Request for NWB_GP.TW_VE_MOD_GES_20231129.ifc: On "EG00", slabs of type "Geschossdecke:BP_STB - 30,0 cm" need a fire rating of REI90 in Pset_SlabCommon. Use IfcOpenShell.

First a look at what the model holds.

```python
import ifcopenshell
import ifcopenshell.util.element

model = ifcopenshell.open("NWB_GP.TW_VE_MOD_GES_20231129.ifc")
print(model.schema)
storey = next(s for s in model.by_type("IfcBuildingStorey") if s.Name == "EG00")
slabs = [e for e in ifcopenshell.util.element.get_decomposition(storey) if e.is_a("IfcSlab")]
seen = {}
for e in slabs:
    element_type = ifcopenshell.util.element.get_type(e)
    key = (element_type.Name if element_type != e and element_type else None, ifcopenshell.util.element.get_pset(e, "Pset_SlabCommon", "FireRating"))
    seen[key] = seen.get(key, 0) + 1
for (name, value), count in sorted(seen.items(), key=str):
    print(count, "x", name, "|", value)
```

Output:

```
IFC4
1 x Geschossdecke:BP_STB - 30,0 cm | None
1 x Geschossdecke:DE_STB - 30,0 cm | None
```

```python
import ifcopenshell
import ifcopenshell.api.pset
import ifcopenshell.util.element

model = ifcopenshell.open("NWB_GP.TW_VE_MOD_GES_20231129.ifc")

storey = next(s for s in model.by_type("IfcBuildingStorey") if s.Name == "EG00")
slabs = [e for e in ifcopenshell.util.element.get_decomposition(storey) if e.is_a("IfcSlab")]

count = 0
for e in slabs:
    element_type = ifcopenshell.util.element.get_type(e)
    if element_type in (None, e) or element_type.Name != "Geschossdecke:BP_STB - 30,0 cm":
        continue
    # add_pset returns the element's existing set when there is one.
    pset = ifcopenshell.api.pset.add_pset(model, product=e, name="Pset_SlabCommon")
    ifcopenshell.api.pset.edit_pset(model, pset=pset, properties={"FireRating": "REI90"})
    count += 1

print(count, "slabs updated")

model.write("NWB_GP.TW_VE_MOD_GES_20231129-out.ifc")
```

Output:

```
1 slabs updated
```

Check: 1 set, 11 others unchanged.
